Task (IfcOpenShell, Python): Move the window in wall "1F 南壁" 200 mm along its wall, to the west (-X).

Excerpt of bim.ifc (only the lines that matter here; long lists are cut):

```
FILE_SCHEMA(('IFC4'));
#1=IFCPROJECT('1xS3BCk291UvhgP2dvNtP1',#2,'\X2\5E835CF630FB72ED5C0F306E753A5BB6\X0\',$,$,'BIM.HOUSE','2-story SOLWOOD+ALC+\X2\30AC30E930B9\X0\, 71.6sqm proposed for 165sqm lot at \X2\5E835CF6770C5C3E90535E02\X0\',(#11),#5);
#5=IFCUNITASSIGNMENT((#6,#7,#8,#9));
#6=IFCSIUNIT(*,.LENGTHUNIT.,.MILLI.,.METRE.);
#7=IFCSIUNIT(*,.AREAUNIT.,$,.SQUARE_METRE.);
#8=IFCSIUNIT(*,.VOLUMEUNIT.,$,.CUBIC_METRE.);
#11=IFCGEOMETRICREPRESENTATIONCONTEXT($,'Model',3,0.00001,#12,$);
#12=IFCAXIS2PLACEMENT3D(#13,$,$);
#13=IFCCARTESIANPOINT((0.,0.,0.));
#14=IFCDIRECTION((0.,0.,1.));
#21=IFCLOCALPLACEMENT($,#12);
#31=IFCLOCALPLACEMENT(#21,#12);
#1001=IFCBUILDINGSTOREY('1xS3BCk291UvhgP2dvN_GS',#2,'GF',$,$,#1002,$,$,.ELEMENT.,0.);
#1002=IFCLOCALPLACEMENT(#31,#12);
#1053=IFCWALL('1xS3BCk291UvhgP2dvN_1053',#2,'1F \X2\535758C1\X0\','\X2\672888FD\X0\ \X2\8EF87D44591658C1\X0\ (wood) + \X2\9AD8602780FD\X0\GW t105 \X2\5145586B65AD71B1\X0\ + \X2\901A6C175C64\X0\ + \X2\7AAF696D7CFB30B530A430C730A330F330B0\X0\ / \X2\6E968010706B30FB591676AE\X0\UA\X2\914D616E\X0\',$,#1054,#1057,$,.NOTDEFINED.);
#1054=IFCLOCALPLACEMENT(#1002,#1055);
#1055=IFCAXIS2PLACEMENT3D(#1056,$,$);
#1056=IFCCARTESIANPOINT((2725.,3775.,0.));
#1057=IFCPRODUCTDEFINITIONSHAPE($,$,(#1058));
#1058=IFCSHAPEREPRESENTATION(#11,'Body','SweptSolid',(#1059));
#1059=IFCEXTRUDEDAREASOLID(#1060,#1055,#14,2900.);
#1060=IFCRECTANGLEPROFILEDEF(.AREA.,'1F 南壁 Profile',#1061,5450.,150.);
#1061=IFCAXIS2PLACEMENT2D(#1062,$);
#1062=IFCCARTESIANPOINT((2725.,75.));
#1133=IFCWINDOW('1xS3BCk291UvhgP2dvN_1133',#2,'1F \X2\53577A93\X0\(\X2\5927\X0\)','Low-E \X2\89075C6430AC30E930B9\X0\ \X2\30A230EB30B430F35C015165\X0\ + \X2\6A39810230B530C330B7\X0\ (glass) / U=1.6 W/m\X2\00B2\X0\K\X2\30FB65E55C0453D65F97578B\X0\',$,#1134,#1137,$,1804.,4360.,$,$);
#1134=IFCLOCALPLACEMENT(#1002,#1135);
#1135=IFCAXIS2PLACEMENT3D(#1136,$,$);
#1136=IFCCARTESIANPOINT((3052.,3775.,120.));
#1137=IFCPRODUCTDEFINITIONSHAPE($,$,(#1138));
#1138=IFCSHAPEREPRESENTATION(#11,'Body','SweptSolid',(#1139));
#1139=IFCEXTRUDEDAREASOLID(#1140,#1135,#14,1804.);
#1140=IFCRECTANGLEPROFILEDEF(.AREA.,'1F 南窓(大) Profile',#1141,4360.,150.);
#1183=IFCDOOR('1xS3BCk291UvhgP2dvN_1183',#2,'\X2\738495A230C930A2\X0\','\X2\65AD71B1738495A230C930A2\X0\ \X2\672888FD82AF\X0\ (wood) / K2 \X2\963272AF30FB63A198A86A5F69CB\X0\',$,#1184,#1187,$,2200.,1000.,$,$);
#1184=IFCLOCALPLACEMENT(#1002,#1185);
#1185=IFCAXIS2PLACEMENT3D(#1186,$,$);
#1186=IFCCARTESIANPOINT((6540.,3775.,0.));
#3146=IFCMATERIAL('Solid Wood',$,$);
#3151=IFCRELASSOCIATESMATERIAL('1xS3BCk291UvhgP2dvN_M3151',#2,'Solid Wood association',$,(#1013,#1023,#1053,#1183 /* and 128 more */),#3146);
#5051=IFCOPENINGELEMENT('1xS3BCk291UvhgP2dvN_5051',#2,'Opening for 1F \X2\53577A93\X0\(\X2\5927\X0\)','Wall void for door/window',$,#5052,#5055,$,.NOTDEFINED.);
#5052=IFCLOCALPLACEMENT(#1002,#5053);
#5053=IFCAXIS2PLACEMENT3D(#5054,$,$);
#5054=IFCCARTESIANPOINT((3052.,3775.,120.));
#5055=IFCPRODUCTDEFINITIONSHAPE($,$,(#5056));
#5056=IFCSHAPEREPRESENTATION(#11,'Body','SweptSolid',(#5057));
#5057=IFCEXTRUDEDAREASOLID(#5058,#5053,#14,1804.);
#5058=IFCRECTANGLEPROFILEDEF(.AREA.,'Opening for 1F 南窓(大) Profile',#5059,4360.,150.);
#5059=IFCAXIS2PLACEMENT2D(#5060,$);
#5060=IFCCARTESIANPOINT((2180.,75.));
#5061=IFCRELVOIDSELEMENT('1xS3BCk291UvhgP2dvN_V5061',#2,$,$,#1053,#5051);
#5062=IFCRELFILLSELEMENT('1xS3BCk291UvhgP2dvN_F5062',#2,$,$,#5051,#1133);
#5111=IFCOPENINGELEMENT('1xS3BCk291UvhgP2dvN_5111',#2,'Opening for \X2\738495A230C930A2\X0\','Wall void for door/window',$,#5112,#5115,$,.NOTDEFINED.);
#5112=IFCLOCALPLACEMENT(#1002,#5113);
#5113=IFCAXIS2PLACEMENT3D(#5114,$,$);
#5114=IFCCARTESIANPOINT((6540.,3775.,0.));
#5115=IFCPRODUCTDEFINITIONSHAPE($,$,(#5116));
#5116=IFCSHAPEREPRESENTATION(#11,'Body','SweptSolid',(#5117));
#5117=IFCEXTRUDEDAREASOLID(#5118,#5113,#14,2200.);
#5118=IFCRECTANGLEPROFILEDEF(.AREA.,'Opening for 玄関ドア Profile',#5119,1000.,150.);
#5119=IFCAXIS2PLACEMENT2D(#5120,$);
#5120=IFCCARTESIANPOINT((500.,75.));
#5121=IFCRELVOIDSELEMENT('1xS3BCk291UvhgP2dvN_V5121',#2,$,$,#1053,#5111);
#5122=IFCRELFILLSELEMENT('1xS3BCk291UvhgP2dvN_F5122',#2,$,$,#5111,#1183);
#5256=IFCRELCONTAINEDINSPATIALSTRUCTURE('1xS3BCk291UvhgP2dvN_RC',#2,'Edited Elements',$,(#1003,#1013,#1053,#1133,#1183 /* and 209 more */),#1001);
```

```python
import ifcopenshell
import ifcopenshell.api.geometry
import ifcopenshell.util.placement

model = ifcopenshell.open("bim.ifc")

window = model.by_id(1133)
opening = window.FillsVoids[0].RelatingOpeningElement
wall = opening.VoidsElements[0].RelatingBuildingElement

wall_matrix = ifcopenshell.util.placement.get_local_placement(wall.ObjectPlacement)
shift = wall_matrix[:3, 0] * -200.0
before = ifcopenshell.util.placement.get_local_placement(window.ObjectPlacement)[:3, 3].copy()

# The window is not placed relative to its opening, so move both.
for product in (opening, window):
    matrix = ifcopenshell.util.placement.get_local_placement(product.ObjectPlacement)
    matrix[:3, 3] += shift
    ifcopenshell.api.geometry.edit_object_placement(model, product=product, matrix=matrix, is_si=False)

after = ifcopenshell.util.placement.get_local_placement(window.ObjectPlacement)[:3, 3]
print("window moved by", (after - before).round(3) + 0.0)

model.write("bim-out.ifc")
```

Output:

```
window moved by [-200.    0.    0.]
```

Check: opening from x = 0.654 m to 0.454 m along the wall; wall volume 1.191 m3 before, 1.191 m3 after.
